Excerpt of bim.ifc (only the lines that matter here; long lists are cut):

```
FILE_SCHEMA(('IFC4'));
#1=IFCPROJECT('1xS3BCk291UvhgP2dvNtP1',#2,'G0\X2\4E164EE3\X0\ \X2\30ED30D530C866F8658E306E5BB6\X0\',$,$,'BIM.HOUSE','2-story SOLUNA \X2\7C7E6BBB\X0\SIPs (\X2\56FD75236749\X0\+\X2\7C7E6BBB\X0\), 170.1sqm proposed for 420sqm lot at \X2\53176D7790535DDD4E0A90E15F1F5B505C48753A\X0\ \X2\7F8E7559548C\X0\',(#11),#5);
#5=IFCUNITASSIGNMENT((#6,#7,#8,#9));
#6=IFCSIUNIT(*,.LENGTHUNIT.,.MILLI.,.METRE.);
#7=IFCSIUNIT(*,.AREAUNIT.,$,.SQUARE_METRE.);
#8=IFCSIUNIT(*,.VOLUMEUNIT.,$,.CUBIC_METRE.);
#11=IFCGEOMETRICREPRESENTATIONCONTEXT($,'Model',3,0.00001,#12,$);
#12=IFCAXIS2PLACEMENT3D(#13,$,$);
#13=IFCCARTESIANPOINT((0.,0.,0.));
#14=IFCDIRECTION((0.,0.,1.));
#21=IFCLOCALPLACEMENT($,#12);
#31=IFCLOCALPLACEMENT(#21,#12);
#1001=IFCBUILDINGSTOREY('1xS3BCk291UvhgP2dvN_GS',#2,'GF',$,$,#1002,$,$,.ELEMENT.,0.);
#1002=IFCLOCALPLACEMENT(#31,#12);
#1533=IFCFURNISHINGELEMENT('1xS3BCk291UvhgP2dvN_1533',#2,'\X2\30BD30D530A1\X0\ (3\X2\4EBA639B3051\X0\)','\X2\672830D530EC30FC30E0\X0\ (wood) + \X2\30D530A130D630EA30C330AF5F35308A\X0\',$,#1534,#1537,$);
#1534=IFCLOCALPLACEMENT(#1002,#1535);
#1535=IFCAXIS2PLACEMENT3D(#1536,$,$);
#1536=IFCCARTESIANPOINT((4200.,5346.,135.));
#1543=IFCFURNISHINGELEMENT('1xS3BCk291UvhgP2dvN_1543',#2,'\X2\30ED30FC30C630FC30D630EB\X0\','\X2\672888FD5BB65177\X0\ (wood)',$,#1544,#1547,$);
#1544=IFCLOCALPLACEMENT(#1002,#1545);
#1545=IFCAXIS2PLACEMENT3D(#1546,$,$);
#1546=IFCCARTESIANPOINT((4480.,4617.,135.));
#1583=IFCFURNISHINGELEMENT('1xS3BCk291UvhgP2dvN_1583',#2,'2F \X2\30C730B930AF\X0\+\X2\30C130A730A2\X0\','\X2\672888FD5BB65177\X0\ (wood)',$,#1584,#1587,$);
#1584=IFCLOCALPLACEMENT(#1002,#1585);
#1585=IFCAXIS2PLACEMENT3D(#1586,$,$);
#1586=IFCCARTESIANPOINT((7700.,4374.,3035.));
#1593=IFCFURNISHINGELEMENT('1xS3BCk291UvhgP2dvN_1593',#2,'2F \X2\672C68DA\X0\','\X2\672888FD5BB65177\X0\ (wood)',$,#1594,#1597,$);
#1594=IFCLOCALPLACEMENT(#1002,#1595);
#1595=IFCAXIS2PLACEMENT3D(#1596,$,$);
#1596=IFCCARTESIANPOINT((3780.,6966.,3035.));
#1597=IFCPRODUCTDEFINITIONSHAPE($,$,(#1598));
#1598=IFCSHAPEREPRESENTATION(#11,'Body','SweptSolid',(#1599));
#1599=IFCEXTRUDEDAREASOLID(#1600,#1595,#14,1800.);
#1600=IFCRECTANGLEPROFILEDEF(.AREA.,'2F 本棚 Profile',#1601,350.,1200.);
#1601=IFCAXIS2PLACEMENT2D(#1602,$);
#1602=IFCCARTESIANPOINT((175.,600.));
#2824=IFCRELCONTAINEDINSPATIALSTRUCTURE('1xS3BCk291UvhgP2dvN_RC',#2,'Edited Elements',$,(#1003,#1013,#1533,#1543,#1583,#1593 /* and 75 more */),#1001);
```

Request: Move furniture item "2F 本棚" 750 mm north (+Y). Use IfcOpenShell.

```python
import ifcopenshell
import ifcopenshell.api.geometry
import ifcopenshell.util.placement
import ifcopenshell.util.unit

model = ifcopenshell.open("bim.ifc")
unit_scale = ifcopenshell.util.unit.calculate_unit_scale(model)

item = model.by_guid("1xS3BCk291UvhgP2dvN_1593")
matrix = ifcopenshell.util.placement.get_local_placement(item.ObjectPlacement)
matrix[1, 3] += 0.75 / unit_scale
ifcopenshell.api.geometry.edit_object_placement(model, product=item, matrix=matrix, is_si=False)

print(ifcopenshell.util.placement.get_local_placement(item.ObjectPlacement).round(3) + 0.0)

model.write("bim_v2.ifc")
```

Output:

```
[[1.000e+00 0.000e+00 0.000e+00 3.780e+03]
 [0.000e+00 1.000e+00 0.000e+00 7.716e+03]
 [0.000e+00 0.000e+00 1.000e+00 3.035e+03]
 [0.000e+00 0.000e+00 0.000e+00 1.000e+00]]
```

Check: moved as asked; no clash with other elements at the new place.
